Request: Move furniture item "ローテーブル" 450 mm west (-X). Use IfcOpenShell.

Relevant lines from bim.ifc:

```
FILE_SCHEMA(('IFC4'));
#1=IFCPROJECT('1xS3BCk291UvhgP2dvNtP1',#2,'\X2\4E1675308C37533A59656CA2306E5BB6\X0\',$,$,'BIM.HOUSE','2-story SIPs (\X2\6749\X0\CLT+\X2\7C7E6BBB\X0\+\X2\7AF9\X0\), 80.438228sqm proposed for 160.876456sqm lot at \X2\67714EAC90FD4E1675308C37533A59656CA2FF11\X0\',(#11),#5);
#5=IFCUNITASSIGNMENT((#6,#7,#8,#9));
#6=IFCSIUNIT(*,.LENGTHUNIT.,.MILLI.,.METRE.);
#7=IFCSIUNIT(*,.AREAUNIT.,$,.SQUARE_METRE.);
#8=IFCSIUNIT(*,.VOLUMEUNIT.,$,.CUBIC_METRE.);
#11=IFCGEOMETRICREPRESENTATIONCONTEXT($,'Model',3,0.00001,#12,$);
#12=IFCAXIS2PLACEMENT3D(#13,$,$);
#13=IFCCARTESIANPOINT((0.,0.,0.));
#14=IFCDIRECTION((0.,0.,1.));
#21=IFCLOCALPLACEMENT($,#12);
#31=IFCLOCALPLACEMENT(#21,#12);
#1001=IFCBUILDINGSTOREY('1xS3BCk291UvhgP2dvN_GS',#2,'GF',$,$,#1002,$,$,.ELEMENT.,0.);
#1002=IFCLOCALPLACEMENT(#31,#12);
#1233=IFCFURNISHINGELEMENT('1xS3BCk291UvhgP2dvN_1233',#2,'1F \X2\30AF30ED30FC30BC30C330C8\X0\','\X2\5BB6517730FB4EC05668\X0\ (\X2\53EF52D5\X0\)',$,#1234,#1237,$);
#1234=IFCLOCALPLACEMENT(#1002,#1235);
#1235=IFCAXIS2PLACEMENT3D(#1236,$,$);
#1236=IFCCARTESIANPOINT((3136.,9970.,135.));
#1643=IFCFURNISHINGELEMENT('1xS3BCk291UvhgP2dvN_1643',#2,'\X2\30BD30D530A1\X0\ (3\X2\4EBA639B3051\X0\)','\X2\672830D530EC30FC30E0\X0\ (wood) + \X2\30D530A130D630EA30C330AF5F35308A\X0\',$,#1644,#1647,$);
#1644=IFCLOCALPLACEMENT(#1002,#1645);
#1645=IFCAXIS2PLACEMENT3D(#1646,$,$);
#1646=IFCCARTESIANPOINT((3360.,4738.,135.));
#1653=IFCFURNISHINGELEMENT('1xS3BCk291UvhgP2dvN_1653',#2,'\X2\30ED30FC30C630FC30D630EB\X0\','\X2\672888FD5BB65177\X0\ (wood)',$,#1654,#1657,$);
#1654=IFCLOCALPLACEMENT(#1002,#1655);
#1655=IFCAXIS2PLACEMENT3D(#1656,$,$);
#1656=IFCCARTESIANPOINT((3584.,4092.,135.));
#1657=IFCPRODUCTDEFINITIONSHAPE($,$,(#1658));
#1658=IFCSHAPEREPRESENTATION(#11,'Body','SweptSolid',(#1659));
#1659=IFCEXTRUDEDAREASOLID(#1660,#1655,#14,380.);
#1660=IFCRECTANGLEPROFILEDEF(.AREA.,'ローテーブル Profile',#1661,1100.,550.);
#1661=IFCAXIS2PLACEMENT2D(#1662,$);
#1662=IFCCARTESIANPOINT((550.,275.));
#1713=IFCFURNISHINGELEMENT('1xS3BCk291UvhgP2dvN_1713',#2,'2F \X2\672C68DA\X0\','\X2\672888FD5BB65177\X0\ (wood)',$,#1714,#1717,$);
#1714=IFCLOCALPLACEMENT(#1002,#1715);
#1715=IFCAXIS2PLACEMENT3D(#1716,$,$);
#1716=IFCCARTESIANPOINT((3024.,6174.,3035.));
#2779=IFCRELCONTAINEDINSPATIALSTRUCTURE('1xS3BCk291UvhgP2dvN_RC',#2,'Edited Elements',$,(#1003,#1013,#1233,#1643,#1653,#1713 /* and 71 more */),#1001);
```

```python
import ifcopenshell
import ifcopenshell.api.geometry
import ifcopenshell.util.placement
import ifcopenshell.util.unit

model = ifcopenshell.open("bim.ifc")
unit_scale = ifcopenshell.util.unit.calculate_unit_scale(model)

item = model.by_guid("1xS3BCk291UvhgP2dvN_1653")
matrix = ifcopenshell.util.placement.get_local_placement(item.ObjectPlacement)
matrix[0, 3] -= 0.45 / unit_scale
ifcopenshell.api.geometry.edit_object_placement(model, product=item, matrix=matrix, is_si=False)

print(ifcopenshell.util.placement.get_local_placement(item.ObjectPlacement).round(3) + 0.0)

model.write("bim-out.ifc")
```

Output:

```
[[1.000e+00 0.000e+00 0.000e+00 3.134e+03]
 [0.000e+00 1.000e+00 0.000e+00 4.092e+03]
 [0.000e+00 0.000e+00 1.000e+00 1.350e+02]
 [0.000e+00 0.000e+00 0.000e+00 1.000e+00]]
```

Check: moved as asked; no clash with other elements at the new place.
